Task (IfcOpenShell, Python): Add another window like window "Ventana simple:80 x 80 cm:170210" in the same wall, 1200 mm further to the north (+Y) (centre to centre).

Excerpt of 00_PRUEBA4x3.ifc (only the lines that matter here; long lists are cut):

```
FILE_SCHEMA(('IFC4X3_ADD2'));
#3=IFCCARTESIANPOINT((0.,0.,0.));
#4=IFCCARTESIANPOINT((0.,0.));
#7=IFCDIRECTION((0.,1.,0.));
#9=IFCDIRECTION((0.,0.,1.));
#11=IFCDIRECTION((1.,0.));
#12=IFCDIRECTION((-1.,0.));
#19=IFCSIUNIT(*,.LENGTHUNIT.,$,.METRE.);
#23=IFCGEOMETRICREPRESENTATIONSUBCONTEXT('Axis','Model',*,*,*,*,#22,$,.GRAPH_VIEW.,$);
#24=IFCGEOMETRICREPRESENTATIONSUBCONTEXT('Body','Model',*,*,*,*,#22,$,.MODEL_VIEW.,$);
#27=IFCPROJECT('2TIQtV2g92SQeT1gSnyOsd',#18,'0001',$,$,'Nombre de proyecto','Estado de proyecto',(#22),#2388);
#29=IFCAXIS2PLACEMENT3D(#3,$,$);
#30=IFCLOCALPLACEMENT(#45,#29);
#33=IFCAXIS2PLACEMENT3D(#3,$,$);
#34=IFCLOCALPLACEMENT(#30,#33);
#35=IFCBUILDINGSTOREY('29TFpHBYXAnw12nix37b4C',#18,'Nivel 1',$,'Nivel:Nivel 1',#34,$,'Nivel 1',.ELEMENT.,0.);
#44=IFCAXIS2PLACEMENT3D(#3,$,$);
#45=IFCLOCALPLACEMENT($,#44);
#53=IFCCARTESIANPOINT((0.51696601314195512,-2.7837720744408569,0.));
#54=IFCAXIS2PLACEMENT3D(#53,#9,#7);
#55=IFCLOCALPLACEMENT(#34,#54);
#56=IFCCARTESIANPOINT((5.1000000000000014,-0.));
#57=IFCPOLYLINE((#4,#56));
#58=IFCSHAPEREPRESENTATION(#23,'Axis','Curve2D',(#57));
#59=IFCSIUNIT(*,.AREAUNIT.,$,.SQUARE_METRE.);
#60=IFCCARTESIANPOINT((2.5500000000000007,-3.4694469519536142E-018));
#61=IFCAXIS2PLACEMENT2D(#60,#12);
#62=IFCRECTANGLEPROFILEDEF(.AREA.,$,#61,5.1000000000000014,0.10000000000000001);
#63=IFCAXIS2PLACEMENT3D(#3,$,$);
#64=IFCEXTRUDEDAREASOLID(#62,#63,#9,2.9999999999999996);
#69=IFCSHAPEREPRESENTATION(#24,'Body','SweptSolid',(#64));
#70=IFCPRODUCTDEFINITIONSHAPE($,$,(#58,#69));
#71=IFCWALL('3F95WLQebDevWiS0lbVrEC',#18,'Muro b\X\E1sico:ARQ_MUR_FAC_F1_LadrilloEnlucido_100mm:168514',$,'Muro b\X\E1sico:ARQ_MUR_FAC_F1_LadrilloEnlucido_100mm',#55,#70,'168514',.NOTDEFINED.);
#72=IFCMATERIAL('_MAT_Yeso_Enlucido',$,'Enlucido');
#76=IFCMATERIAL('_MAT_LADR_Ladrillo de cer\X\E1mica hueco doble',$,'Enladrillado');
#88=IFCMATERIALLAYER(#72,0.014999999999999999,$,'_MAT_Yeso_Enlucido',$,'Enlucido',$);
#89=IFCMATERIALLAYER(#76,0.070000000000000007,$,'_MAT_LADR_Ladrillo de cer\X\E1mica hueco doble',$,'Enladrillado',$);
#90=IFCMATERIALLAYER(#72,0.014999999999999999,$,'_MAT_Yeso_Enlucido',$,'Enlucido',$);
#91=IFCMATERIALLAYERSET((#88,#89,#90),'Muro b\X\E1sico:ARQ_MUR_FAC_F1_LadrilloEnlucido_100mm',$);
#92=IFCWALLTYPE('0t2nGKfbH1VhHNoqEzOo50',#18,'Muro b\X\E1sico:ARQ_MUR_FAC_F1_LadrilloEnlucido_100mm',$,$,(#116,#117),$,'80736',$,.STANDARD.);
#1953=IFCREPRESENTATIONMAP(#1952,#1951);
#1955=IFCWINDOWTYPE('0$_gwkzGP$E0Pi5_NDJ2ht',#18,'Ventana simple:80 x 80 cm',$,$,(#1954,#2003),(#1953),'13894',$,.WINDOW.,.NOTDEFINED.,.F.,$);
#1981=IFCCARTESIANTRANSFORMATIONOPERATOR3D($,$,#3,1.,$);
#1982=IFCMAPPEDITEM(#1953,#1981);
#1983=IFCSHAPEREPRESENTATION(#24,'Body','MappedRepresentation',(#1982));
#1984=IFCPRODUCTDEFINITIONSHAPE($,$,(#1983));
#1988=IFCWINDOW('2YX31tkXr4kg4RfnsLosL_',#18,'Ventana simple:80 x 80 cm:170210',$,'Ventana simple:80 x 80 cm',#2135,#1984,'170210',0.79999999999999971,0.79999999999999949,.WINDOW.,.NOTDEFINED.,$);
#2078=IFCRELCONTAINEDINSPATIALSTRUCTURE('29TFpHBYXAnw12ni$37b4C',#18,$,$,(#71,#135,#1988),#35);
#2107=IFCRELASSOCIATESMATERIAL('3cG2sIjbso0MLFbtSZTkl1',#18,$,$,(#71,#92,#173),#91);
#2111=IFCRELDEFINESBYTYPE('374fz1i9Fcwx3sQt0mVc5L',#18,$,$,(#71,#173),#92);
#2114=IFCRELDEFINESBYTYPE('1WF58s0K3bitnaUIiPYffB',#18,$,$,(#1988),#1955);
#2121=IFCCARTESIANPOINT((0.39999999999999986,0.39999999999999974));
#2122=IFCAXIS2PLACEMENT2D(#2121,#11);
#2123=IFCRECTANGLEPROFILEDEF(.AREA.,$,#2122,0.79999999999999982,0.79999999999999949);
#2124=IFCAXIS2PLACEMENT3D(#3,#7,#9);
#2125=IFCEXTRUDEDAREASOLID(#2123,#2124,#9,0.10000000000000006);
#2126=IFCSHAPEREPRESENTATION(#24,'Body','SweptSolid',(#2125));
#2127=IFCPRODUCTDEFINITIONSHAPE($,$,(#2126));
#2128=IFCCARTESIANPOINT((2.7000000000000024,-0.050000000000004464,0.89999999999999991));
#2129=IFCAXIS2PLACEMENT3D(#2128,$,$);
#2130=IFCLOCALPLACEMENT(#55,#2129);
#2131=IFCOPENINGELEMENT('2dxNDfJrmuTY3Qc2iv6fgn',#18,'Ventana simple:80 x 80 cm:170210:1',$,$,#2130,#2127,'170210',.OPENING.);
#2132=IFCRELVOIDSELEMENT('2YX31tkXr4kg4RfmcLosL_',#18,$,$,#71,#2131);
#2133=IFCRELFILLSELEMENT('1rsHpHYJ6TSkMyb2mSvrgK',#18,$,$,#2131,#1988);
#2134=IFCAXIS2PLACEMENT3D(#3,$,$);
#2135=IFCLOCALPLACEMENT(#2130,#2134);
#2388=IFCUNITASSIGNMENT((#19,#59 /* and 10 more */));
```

```python
import ifcopenshell
import ifcopenshell.api.feature
import ifcopenshell.api.geometry
import ifcopenshell.api.root
import ifcopenshell.geom
import ifcopenshell.util.element
import ifcopenshell.util.placement
import ifcopenshell.util.shape

model = ifcopenshell.open("00_PRUEBA4x3.ifc")
settings = ifcopenshell.geom.settings()


def volume(element):
    """Net volume in cubic metres, openings subtracted."""
    shape = ifcopenshell.geom.create_shape(settings, element)
    return ifcopenshell.util.shape.get_volume(shape.geometry)


def reuse_history(source, copy):
    """copy_class also copies each property set's owner history, people and application; keep the originals."""
    for rel in copy.IsDefinedBy:
        if rel.is_a("IfcRelDefinesByProperties") and (history := rel.RelatingPropertyDefinition.OwnerHistory):
            rel.RelatingPropertyDefinition.OwnerHistory = source.OwnerHistory
            ifcopenshell.util.element.remove_deep2(model, history)


window = model.by_guid("2YX31tkXr4kg4RfnsLosL_")
opening = window.FillsVoids[0].RelatingOpeningElement
wall = opening.VoidsElements[0].RelatingBuildingElement
before = volume(wall)
shift = ifcopenshell.util.placement.get_local_placement(wall.ObjectPlacement)[:3, 0] * 1.2

# copy_class copies the void relationship, type, container and properties, but no geometry.
new_opening = ifcopenshell.api.root.copy_class(model, product=opening)
new_opening.Representation = ifcopenshell.util.element.copy_deep(
    model, opening.Representation, exclude=["IfcGeometricRepresentationContext", "IfcRepresentationMap"]
)
new_opening.Name = "Ventana simple:80 x 80 cm"
new_opening.Tag = None
new_window = ifcopenshell.api.root.copy_class(model, product=window)
new_window.Representation = ifcopenshell.util.element.copy_deep(
    model, window.Representation, exclude=["IfcGeometricRepresentationContext", "IfcRepresentationMap"]
)
new_window.Name = "Ventana simple:80 x 80 cm"
new_window.Tag = None
reuse_history(window, new_window)
ifcopenshell.api.feature.add_filling(model, opening=new_opening, element=new_window)

for old, new in ((opening, new_opening), (window, new_window)):
    matrix = ifcopenshell.util.placement.get_local_placement(old.ObjectPlacement)
    matrix[:3, 3] += shift
    ifcopenshell.api.geometry.edit_object_placement(model, product=new, matrix=matrix, is_si=False)

after = volume(wall)

print(f"wall volume {before:.3f} -> {after:.3f} m3")

model.write("00_PRUEBA4x3_rev.ifc")
```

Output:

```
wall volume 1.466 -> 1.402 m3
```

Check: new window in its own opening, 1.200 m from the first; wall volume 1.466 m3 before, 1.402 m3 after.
